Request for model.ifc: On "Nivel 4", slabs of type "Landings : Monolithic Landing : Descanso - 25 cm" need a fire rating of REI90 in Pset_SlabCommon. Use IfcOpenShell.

First a look at what the model holds.

```python
import ifcopenshell
import ifcopenshell.util.element

model = ifcopenshell.open("model.ifc")
print(model.schema)
storey = next(s for s in model.by_type("IfcBuildingStorey") if s.Name == "Nivel 4")
slabs = [e for e in ifcopenshell.util.element.get_decomposition(storey) if e.is_a("IfcSlab")]
seen = {}
for e in slabs:
    element_type = ifcopenshell.util.element.get_type(e)
    key = (element_type.Name if element_type != e and element_type else None, ifcopenshell.util.element.get_pset(e, "Pset_SlabCommon", "FireRating"))
    seen[key] = seen.get(key, 0) + 1
for (name, value), count in sorted(seen.items(), key=str):
    print(count, "x", name, "|", value)
```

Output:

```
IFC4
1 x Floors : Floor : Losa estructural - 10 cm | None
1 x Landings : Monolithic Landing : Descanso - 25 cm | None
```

```python
import ifcopenshell
import ifcopenshell.api.pset
import ifcopenshell.util.element

model = ifcopenshell.open("model.ifc")

storey = next(s for s in model.by_type("IfcBuildingStorey") if s.Name == "Nivel 4")
slabs = [e for e in ifcopenshell.util.element.get_decomposition(storey) if e.is_a("IfcSlab")]

count = 0
for e in slabs:
    element_type = ifcopenshell.util.element.get_type(e)
    if element_type in (None, e) or element_type.Name != "Landings : Monolithic Landing : Descanso - 25 cm":
        continue
    # add_pset returns the element's existing set when there is one.
    pset = ifcopenshell.api.pset.add_pset(model, product=e, name="Pset_SlabCommon")
    ifcopenshell.api.pset.edit_pset(model, pset=pset, properties={"FireRating": "REI90"})
    count += 1

print(count, "slabs updated")

model.write("model_edited.ifc")
```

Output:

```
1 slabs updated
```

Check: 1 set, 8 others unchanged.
